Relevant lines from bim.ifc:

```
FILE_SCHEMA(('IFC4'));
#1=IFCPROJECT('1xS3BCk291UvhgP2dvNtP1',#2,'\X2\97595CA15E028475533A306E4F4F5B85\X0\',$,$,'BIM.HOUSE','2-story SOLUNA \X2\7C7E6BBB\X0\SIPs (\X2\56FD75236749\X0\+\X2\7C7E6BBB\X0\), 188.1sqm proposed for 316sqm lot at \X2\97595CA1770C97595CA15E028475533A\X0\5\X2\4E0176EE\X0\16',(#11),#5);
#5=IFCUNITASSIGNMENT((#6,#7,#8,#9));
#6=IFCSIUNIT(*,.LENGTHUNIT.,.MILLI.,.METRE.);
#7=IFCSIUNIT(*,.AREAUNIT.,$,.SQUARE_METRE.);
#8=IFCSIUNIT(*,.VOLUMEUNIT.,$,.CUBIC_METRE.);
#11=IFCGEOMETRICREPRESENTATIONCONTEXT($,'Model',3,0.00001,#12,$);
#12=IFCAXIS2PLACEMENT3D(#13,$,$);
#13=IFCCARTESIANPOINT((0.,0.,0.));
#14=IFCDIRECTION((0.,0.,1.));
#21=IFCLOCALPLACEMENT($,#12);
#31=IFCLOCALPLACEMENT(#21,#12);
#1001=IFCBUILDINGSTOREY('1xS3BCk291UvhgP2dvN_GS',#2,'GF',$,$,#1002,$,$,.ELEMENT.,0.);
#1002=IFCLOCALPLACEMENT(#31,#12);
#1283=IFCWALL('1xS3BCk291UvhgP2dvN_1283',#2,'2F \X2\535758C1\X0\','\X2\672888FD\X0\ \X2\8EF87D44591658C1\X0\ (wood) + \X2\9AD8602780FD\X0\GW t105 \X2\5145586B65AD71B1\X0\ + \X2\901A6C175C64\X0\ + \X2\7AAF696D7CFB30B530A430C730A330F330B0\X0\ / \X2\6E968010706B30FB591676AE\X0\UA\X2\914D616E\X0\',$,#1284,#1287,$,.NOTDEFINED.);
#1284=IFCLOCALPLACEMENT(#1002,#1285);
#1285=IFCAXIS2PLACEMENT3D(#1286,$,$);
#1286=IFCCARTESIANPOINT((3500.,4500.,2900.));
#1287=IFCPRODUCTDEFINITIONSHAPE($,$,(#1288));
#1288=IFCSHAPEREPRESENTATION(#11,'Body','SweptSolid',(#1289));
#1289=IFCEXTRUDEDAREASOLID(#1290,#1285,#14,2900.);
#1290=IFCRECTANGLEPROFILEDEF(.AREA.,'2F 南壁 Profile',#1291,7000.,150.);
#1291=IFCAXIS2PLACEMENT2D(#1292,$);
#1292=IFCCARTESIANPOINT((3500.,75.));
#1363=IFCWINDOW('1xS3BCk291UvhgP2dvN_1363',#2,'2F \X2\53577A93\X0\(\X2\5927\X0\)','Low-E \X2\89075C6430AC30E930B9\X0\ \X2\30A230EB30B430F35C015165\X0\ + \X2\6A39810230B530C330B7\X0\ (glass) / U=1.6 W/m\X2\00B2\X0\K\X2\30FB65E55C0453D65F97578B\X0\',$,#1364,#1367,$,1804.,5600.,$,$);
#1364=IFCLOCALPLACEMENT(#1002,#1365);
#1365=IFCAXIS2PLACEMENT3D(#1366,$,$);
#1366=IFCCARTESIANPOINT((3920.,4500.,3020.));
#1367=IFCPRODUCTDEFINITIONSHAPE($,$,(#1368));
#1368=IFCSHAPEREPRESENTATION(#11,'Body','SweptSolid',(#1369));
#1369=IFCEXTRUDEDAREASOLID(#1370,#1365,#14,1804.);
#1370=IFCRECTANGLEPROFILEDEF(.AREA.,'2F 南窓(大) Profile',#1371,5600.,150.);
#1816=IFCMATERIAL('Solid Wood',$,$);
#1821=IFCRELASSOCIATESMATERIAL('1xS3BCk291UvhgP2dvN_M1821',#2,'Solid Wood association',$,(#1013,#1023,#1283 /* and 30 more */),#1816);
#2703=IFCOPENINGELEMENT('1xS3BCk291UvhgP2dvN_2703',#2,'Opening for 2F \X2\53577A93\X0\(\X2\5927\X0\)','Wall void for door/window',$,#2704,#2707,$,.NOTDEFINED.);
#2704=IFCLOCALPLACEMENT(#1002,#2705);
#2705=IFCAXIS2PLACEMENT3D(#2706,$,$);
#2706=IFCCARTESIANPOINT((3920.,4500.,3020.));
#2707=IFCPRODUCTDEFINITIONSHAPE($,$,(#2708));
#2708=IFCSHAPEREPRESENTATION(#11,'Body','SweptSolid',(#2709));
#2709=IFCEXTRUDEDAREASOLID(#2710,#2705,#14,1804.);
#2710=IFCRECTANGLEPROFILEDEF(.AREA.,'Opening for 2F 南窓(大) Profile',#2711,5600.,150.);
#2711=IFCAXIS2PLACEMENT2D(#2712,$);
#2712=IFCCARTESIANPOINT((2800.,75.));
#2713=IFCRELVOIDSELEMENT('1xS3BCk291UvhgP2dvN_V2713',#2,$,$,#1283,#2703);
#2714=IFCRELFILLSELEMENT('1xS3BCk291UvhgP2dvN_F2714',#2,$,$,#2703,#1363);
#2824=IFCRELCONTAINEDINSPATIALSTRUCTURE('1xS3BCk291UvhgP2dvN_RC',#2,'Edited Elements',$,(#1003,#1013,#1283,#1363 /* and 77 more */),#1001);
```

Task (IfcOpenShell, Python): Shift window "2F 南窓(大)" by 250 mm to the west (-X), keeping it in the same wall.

```python
import ifcopenshell
import ifcopenshell.api.geometry
import ifcopenshell.util.placement
import ifcopenshell.util.unit

model = ifcopenshell.open("bim.ifc")
unit_scale = ifcopenshell.util.unit.calculate_unit_scale(model)

window = model.by_guid("1xS3BCk291UvhgP2dvN_1363")
opening = window.FillsVoids[0].RelatingOpeningElement
wall = opening.VoidsElements[0].RelatingBuildingElement

wall_matrix = ifcopenshell.util.placement.get_local_placement(wall.ObjectPlacement)
shift = wall_matrix[:3, 0] * -0.25 / unit_scale
before = ifcopenshell.util.placement.get_local_placement(window.ObjectPlacement)[:3, 3].copy()

# The window is not placed relative to its opening, so move both.
for product in (opening, window):
    matrix = ifcopenshell.util.placement.get_local_placement(product.ObjectPlacement)
    matrix[:3, 3] += shift
    ifcopenshell.api.geometry.edit_object_placement(model, product=product, matrix=matrix, is_si=False)

after = ifcopenshell.util.placement.get_local_placement(window.ObjectPlacement)[:3, 3]
print("window moved by", (after - before).round(3) + 0.0)

model.write("bim_updated.ifc")
```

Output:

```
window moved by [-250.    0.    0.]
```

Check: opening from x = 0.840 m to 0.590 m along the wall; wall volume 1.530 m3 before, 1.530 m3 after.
